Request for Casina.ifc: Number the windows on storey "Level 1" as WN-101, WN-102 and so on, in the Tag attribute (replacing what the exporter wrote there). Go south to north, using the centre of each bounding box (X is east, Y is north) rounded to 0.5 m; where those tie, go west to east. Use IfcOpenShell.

First a look at what the model holds.

```python
import ifcopenshell
import ifcopenshell.util.element
import ifcopenshell.util.placement

model = ifcopenshell.open("Casina.ifc")
print(model.schema)
storey = next(s for s in model.by_type("IfcBuildingStorey") if s.Name == "Level 1")
windows = [e for e in ifcopenshell.util.element.get_decomposition(storey) if e.is_a("IfcWindow")]
for e in sorted(windows, key=lambda e: e.id()):
    origin = ifcopenshell.util.placement.get_local_placement(e.ObjectPlacement)[:3, 3]
    print(e.id(), e.Tag, e.Name, origin.round(2) + 0.0, sep=" | ")
```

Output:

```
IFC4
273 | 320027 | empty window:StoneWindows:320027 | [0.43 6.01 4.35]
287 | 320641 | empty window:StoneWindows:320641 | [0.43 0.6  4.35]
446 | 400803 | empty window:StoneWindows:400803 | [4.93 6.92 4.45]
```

```python
import ifcopenshell
import ifcopenshell.geom
import ifcopenshell.util.element
import ifcopenshell.util.shape

model = ifcopenshell.open("Casina.ifc")
settings = ifcopenshell.geom.settings()
settings.set("use-world-coords", True)


def centre(element):
    shape = ifcopenshell.geom.create_shape(settings, element)
    return ifcopenshell.util.shape.get_bbox_centroid(shape.geometry)


storey = next(s for s in model.by_type("IfcBuildingStorey") if s.Name == "Level 1")
windows = [e for e in ifcopenshell.util.element.get_decomposition(storey) if e.is_a("IfcWindow")]

# Insertion points can sit at a corner or the storey origin, so sort by the geometry (in metres).
centres = {e: centre(e) for e in windows}
windows.sort(key=lambda e: (round(centres[e][1] / 0.5), centres[e][0]))

for i, e in enumerate(windows, start=1):
    number = f"WN-1{i:02d}"
    e.Tag = number
    print(e.id(), number)

model.write("Casina-out.ifc")
```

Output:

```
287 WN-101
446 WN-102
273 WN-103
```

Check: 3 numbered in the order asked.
